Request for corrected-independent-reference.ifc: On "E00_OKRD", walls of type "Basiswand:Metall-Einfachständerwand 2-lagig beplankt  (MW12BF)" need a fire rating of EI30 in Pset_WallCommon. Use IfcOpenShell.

First a look at what the model holds.

```python
import ifcopenshell
import ifcopenshell.util.element

model = ifcopenshell.open("corrected-independent-reference.ifc")
print(model.schema)
storey = next(s for s in model.by_type("IfcBuildingStorey") if s.Name == "E00_OKRD")
walls = [e for e in ifcopenshell.util.element.get_decomposition(storey) if e.is_a("IfcWall")]
seen = {}
for e in walls:
    element_type = ifcopenshell.util.element.get_type(e)
    key = (element_type.Name if element_type != e and element_type else None, ifcopenshell.util.element.get_pset(e, "Pset_WallCommon", "FireRating"))
    seen[key] = seen.get(key, 0) + 1
for (name, value), count in sorted(seen.items(), key=str):
    print(count, "x", name, "|", value)
```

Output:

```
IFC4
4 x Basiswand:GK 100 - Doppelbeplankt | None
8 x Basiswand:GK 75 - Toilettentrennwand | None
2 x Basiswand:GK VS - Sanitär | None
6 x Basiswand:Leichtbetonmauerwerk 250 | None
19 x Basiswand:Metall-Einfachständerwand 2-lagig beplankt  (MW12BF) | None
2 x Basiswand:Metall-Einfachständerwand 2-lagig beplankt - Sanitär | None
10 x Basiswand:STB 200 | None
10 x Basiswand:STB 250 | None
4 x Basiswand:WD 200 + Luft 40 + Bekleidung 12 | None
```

```python
import ifcopenshell
import ifcopenshell.api.pset
import ifcopenshell.util.element

model = ifcopenshell.open("corrected-independent-reference.ifc")

storey = next(s for s in model.by_type("IfcBuildingStorey") if s.Name == "E00_OKRD")
walls = [e for e in ifcopenshell.util.element.get_decomposition(storey) if e.is_a("IfcWall")]

count = 0
for e in walls:
    element_type = ifcopenshell.util.element.get_type(e)
    if element_type in (None, e) or element_type.Name != "Basiswand:Metall-Einfachständerwand 2-lagig beplankt  (MW12BF)":
        continue
    # add_pset returns the element's existing set when there is one.
    pset = ifcopenshell.api.pset.add_pset(model, product=e, name="Pset_WallCommon")
    ifcopenshell.api.pset.edit_pset(model, pset=pset, properties={"FireRating": "EI30"})
    count += 1

print(count, "walls updated")

model.write("corrected-independent-reference_v2.ifc")
```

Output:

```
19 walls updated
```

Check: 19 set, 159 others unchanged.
